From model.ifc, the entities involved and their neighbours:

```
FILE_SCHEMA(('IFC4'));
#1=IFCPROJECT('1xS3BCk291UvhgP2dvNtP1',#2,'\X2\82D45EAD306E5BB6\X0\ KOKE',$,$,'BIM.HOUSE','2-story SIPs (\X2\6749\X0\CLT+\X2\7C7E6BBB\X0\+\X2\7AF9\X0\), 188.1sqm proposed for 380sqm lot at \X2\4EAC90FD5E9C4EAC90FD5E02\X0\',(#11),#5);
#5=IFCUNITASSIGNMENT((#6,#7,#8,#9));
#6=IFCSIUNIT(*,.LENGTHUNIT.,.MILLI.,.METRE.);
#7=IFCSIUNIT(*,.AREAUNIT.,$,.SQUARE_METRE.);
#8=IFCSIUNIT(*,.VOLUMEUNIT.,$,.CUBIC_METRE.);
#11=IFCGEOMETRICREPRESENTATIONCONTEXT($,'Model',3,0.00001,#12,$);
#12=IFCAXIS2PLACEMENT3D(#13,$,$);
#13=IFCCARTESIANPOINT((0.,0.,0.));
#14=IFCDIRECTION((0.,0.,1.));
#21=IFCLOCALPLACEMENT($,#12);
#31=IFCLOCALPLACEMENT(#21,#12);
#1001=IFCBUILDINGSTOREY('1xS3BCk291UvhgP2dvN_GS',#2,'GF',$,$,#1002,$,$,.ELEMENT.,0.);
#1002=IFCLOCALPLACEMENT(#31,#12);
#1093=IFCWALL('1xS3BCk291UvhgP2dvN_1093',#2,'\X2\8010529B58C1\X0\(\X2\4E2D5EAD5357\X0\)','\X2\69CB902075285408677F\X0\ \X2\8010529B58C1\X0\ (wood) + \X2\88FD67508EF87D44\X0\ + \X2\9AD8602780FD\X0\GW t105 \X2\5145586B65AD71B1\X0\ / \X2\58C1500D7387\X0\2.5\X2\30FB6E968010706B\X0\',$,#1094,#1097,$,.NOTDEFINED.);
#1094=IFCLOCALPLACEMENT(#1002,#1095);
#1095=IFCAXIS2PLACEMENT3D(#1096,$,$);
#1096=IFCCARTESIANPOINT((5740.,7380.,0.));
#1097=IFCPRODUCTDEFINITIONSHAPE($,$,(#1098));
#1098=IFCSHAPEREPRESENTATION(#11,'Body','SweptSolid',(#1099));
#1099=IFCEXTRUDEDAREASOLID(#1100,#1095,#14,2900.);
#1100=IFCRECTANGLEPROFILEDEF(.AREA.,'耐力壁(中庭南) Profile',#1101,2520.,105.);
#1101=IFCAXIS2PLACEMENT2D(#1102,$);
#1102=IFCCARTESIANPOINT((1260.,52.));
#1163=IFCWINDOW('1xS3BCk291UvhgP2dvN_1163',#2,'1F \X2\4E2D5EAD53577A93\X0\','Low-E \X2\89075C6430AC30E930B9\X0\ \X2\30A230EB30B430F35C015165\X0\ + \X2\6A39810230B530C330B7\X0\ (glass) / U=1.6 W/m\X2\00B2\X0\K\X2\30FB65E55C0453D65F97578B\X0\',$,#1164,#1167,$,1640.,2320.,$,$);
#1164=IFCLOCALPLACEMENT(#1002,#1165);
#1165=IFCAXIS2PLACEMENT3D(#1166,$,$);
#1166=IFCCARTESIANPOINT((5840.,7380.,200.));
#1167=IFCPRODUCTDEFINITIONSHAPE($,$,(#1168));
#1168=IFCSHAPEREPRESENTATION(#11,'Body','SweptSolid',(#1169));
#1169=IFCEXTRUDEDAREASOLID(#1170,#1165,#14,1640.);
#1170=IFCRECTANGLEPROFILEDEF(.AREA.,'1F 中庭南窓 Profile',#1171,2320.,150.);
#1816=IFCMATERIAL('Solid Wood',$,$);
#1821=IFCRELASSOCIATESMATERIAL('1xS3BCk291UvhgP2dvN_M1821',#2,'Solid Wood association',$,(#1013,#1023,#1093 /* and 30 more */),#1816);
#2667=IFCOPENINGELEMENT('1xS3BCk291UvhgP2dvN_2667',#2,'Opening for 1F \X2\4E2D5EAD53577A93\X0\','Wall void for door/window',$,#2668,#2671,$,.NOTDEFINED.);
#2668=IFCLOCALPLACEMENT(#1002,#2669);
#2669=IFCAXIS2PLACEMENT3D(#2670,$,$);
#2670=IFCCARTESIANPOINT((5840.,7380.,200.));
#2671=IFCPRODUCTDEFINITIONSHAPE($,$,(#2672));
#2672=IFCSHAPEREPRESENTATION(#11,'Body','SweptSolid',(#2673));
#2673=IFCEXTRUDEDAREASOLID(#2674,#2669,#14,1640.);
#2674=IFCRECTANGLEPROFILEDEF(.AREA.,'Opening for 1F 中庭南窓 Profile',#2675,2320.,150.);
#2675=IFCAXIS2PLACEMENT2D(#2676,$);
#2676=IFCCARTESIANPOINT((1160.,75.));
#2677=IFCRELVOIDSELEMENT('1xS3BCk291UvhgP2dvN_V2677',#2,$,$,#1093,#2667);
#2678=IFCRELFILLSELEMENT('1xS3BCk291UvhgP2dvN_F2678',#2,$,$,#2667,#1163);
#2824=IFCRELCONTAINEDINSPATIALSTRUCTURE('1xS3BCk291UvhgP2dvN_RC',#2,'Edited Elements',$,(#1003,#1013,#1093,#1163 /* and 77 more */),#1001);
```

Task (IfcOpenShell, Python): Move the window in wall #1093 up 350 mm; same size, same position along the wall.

```python
import numpy as np
import ifcopenshell
import ifcopenshell.api.geometry
import ifcopenshell.util.placement
import ifcopenshell.util.unit

model = ifcopenshell.open("model.ifc")
unit_scale = ifcopenshell.util.unit.calculate_unit_scale(model)

window = model.by_guid("1xS3BCk291UvhgP2dvN_1163")
opening = window.FillsVoids[0].RelatingOpeningElement
dz = 0.35 / unit_scale

shift = np.array([0.0, 0.0, dz])
# The window is not placed relative to its opening, so move both.
for product in (opening, window):
    matrix = ifcopenshell.util.placement.get_local_placement(product.ObjectPlacement)
    matrix[:3, 3] += shift
    ifcopenshell.api.geometry.edit_object_placement(model, product=product, matrix=matrix, is_si=False)

print(f"moved by {dz * unit_scale:+.3f} m")

model.write("model-out.ifc")
```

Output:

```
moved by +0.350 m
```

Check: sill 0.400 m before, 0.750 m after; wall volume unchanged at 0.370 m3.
